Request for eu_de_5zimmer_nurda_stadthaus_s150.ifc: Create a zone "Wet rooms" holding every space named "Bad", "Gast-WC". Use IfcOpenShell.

First a look at what the model holds.

```python
import ifcopenshell

model = ifcopenshell.open("eu_de_5zimmer_nurda_stadthaus_s150.ifc")
print(model.schema)
seen = {}
for space in model.by_type("IfcSpace"):
    seen[space.LongName] = seen.get(space.LongName, 0) + 1
for name, count in sorted(seen.items(), key=str):
    print(count, "x", name)
print("zones:", [z.Name for z in model.by_type("IfcZone")][:20])
```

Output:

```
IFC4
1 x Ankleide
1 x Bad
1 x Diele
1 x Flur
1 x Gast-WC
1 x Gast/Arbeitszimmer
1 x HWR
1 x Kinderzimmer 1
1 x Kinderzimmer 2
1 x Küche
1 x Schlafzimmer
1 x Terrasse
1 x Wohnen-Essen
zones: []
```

```python
import ifcopenshell
import ifcopenshell.api.group
import ifcopenshell.api.root

model = ifcopenshell.open("eu_de_5zimmer_nurda_stadthaus_s150.ifc")

names = {"Bad", "Gast-WC"}
spaces = [s for s in model.by_type("IfcSpace") if s.LongName in names]

zone = ifcopenshell.api.root.create_entity(model, ifc_class="IfcZone", name="Wet rooms")
ifcopenshell.api.group.assign_group(model, products=spaces, group=zone)
print(len(spaces), "spaces in", zone.Name)

model.write("eu_de_5zimmer_nurda_stadthaus_s150_rev.ifc")
```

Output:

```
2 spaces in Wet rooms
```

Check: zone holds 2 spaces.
